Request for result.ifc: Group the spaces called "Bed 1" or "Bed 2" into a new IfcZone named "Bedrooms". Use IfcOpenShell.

First a look at what the model holds.

```python
import ifcopenshell

model = ifcopenshell.open("result.ifc")
print(model.schema)
seen = {}
for space in model.by_type("IfcSpace"):
    seen[space.Name] = seen.get(space.Name, 0) + 1
for name, count in sorted(seen.items(), key=str):
    print(count, "x", name)
print("zones:", [z.Name for z in model.by_type("IfcZone")][:20])
```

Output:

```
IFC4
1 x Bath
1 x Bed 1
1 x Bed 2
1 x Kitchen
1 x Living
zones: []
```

```python
import ifcopenshell
import ifcopenshell.api.group
import ifcopenshell.api.root

model = ifcopenshell.open("result.ifc")

names = {"Bed 1", "Bed 2"}
spaces = [s for s in model.by_type("IfcSpace") if s.Name in names]

zone = ifcopenshell.api.root.create_entity(model, ifc_class="IfcZone", name="Bedrooms")
ifcopenshell.api.group.assign_group(model, products=spaces, group=zone)
print(len(spaces), "spaces in", zone.Name)

model.write("result_rev.ifc")
```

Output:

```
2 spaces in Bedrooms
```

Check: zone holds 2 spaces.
